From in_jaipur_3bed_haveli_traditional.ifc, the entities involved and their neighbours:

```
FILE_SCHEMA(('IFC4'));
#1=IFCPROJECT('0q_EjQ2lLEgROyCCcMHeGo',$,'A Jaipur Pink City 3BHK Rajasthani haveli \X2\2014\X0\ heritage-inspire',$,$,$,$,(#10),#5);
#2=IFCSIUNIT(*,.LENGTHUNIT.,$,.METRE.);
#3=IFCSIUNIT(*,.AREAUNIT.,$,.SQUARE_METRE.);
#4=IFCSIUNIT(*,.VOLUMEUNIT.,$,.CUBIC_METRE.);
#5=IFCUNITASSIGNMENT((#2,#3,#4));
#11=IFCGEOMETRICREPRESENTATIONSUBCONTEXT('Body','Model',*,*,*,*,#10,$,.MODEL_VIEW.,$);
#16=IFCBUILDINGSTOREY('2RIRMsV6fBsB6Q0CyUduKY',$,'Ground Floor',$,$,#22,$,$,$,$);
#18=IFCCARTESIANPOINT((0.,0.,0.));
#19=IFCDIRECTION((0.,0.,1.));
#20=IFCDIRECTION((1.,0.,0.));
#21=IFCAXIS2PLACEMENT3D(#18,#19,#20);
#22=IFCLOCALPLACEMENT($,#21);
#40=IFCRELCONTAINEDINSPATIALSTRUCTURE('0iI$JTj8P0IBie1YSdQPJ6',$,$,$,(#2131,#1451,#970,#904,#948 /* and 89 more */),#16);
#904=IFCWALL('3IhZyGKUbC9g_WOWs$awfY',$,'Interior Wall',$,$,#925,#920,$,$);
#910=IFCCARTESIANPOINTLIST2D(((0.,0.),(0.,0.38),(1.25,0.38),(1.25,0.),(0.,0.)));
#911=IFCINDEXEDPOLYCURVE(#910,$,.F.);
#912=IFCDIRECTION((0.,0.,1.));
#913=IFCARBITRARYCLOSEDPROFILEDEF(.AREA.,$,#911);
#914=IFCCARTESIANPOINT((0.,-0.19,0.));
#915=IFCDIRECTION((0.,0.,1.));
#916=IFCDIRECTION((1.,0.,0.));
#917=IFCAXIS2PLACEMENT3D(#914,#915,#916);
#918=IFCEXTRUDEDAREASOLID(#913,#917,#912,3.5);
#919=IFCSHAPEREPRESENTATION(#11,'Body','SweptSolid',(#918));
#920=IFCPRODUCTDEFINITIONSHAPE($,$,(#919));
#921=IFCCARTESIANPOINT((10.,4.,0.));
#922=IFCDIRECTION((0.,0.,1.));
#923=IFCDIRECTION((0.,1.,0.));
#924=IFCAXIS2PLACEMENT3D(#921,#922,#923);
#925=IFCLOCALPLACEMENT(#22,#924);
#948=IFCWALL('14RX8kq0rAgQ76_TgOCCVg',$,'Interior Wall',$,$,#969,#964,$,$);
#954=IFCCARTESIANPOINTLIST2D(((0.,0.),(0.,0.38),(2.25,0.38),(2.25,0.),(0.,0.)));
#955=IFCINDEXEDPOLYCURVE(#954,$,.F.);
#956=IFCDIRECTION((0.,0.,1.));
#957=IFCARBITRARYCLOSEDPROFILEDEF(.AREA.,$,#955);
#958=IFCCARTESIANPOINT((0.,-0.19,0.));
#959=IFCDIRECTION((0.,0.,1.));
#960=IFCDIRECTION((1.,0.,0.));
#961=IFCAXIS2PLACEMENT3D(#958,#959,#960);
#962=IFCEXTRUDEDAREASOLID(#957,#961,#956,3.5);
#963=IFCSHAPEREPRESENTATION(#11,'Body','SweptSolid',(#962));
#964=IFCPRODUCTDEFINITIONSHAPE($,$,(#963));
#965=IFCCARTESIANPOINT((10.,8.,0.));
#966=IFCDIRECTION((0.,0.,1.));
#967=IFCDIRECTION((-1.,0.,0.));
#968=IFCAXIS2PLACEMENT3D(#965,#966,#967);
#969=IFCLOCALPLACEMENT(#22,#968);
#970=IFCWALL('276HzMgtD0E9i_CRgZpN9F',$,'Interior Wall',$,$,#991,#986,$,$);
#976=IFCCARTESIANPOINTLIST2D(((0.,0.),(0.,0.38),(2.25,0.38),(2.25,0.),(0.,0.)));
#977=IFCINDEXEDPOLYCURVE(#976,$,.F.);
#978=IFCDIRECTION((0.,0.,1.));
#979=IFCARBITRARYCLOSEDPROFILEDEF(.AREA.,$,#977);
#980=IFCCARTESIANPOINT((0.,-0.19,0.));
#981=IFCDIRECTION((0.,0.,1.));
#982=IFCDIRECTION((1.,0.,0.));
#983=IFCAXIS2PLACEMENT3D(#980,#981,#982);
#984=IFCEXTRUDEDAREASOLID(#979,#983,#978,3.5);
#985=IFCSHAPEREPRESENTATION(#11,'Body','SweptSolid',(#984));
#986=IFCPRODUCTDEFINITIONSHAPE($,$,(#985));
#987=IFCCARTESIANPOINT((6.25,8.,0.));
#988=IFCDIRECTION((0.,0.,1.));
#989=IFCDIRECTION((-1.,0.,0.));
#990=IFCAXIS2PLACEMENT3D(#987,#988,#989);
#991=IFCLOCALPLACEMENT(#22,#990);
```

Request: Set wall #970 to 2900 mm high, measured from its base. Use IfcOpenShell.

```python
import ifcopenshell
import ifcopenshell.geom
import ifcopenshell.util.representation
import ifcopenshell.util.shape
import ifcopenshell.util.unit

model = ifcopenshell.open("in_jaipur_3bed_haveli_traditional.ifc")
unit_scale = ifcopenshell.util.unit.calculate_unit_scale(model)
settings = ifcopenshell.geom.settings()


def volume(element):
    """Net volume in cubic metres, openings subtracted."""
    shape = ifcopenshell.geom.create_shape(settings, element)
    return ifcopenshell.util.shape.get_volume(shape.geometry)


wall = model.by_guid("276HzMgtD0E9i_CRgZpN9F")
before = volume(wall)

body = ifcopenshell.util.representation.get_representation(wall, "Model", "Body")
solid = body.Items[0]
old_height = solid.Depth
solid.Depth = 2.9 / unit_scale
after = volume(wall)

print(f"height {old_height:g} -> {solid.Depth:g}, volume {before:.3f} -> {after:.3f} m3")

model.write("in_jaipur_3bed_haveli_traditional_v2.ifc")
```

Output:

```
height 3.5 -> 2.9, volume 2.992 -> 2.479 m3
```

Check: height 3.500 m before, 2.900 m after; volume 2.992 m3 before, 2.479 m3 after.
